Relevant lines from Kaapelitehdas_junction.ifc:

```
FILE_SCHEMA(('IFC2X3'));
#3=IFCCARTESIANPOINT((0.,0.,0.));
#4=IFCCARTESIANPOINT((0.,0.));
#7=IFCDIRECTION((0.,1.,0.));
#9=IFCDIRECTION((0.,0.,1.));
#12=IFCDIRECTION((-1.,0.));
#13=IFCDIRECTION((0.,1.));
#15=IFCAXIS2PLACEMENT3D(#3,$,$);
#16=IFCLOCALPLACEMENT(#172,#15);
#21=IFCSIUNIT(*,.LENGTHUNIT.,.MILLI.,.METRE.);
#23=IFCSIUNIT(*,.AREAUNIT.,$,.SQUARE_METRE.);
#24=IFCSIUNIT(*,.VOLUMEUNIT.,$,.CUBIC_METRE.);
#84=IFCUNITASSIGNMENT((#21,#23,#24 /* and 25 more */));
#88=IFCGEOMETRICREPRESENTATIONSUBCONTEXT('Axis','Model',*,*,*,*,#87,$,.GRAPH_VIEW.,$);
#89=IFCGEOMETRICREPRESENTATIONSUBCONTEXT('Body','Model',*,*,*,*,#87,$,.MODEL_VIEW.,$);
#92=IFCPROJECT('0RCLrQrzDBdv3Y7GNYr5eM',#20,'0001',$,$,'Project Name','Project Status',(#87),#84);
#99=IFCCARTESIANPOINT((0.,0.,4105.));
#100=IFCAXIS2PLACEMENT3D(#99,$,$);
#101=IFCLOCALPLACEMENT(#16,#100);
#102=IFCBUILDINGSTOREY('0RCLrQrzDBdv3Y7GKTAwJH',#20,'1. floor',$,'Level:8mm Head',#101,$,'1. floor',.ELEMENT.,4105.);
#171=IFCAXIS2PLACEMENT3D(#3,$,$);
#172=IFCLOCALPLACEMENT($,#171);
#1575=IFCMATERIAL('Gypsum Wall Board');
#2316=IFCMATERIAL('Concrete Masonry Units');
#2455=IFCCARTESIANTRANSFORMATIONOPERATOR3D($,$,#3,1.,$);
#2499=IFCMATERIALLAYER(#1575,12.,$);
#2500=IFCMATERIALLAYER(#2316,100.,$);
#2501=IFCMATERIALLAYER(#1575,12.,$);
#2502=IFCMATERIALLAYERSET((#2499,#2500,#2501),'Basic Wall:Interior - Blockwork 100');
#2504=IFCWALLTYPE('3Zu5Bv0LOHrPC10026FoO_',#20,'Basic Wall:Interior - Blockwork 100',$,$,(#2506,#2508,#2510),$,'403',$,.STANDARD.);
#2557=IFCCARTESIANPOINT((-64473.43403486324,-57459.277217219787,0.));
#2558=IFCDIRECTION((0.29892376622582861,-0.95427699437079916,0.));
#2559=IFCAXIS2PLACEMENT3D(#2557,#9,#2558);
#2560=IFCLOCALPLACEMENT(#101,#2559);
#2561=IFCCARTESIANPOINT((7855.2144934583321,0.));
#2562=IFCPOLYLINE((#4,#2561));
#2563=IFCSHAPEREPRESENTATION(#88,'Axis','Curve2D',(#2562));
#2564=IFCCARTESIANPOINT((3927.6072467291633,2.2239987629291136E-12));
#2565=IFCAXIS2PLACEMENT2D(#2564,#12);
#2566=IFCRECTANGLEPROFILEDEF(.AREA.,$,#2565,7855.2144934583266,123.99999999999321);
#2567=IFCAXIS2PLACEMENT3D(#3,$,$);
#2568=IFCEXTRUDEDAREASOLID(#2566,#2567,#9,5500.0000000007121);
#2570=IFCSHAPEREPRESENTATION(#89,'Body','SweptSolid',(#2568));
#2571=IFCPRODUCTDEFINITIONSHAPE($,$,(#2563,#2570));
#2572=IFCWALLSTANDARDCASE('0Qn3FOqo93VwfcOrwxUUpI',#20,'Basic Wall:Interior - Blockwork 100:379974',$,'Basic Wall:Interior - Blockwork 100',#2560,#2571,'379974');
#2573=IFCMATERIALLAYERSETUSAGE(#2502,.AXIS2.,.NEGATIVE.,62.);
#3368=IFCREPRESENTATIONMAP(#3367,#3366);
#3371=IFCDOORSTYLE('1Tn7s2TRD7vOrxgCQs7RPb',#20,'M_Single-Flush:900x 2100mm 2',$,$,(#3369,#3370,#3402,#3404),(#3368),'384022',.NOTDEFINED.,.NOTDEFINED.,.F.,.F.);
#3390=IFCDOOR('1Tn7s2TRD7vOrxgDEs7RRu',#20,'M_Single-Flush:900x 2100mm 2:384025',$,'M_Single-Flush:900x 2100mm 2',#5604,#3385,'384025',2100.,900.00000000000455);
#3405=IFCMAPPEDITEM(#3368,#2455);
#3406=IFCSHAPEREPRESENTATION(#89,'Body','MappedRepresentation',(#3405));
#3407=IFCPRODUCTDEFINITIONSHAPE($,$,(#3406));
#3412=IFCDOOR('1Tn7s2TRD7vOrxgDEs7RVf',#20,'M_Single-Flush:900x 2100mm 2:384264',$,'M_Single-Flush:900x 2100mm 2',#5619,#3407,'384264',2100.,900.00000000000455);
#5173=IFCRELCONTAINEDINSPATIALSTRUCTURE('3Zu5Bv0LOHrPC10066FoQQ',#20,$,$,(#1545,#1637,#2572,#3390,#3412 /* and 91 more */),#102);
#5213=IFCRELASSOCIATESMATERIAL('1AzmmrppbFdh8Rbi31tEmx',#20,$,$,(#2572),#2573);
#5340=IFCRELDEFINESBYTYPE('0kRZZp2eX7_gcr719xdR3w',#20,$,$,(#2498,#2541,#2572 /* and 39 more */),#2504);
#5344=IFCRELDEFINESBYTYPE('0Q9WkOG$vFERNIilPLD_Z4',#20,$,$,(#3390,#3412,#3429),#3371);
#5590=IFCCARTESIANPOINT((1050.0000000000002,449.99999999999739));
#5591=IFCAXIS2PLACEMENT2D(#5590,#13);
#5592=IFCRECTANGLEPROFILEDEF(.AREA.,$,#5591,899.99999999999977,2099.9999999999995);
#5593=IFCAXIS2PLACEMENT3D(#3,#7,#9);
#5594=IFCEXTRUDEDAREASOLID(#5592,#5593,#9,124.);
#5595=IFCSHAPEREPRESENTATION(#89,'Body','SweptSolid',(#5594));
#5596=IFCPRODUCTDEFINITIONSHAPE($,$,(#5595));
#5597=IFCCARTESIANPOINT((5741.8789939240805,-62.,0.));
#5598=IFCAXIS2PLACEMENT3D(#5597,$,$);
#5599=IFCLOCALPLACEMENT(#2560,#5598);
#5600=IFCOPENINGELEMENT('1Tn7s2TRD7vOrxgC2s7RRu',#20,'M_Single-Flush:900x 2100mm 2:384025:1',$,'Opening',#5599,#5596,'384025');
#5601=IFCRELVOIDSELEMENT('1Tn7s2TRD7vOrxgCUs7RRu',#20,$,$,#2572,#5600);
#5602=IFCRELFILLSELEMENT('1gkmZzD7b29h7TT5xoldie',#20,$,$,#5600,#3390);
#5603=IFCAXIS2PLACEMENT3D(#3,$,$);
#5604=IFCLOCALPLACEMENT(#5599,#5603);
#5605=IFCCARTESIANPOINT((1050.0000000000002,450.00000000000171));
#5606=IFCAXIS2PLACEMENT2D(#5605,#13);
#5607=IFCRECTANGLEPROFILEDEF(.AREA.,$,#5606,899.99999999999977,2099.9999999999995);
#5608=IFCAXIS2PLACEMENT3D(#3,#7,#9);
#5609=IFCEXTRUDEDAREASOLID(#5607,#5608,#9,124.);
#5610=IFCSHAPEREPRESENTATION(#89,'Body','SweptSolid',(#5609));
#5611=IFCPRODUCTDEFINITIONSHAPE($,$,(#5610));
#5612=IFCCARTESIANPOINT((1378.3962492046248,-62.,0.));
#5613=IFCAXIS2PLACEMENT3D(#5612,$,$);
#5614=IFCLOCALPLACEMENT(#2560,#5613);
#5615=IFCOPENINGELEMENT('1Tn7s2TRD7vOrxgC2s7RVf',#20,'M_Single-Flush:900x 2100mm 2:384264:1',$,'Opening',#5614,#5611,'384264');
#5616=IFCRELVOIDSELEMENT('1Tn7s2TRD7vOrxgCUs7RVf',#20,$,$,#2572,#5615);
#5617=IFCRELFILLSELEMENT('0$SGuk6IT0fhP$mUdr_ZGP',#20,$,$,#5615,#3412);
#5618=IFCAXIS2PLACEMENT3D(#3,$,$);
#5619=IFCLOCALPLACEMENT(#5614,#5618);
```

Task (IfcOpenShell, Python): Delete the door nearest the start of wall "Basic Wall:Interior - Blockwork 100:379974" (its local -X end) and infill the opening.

```python
import ifcopenshell
import ifcopenshell.api.feature
import ifcopenshell.api.root
import ifcopenshell.geom
import ifcopenshell.util.shape

model = ifcopenshell.open("Kaapelitehdas_junction.ifc")
settings = ifcopenshell.geom.settings()


def volume(element):
    """Net volume in cubic metres, openings subtracted."""
    shape = ifcopenshell.geom.create_shape(settings, element)
    return ifcopenshell.util.shape.get_volume(shape.geometry)


door = model.by_id(3412)
opening = door.FillsVoids[0].RelatingOpeningElement
wall = opening.VoidsElements[0].RelatingBuildingElement
before = volume(wall)

ifcopenshell.api.root.remove_product(model, product=door)
ifcopenshell.api.feature.remove_feature(model, feature=opening)

after = volume(wall)

print(f"wall volume {before:.3f} -> {after:.3f} m3")

model.write("Kaapelitehdas_junction_updated.ifc")
```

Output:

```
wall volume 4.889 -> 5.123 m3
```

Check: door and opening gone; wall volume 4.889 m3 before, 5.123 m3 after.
